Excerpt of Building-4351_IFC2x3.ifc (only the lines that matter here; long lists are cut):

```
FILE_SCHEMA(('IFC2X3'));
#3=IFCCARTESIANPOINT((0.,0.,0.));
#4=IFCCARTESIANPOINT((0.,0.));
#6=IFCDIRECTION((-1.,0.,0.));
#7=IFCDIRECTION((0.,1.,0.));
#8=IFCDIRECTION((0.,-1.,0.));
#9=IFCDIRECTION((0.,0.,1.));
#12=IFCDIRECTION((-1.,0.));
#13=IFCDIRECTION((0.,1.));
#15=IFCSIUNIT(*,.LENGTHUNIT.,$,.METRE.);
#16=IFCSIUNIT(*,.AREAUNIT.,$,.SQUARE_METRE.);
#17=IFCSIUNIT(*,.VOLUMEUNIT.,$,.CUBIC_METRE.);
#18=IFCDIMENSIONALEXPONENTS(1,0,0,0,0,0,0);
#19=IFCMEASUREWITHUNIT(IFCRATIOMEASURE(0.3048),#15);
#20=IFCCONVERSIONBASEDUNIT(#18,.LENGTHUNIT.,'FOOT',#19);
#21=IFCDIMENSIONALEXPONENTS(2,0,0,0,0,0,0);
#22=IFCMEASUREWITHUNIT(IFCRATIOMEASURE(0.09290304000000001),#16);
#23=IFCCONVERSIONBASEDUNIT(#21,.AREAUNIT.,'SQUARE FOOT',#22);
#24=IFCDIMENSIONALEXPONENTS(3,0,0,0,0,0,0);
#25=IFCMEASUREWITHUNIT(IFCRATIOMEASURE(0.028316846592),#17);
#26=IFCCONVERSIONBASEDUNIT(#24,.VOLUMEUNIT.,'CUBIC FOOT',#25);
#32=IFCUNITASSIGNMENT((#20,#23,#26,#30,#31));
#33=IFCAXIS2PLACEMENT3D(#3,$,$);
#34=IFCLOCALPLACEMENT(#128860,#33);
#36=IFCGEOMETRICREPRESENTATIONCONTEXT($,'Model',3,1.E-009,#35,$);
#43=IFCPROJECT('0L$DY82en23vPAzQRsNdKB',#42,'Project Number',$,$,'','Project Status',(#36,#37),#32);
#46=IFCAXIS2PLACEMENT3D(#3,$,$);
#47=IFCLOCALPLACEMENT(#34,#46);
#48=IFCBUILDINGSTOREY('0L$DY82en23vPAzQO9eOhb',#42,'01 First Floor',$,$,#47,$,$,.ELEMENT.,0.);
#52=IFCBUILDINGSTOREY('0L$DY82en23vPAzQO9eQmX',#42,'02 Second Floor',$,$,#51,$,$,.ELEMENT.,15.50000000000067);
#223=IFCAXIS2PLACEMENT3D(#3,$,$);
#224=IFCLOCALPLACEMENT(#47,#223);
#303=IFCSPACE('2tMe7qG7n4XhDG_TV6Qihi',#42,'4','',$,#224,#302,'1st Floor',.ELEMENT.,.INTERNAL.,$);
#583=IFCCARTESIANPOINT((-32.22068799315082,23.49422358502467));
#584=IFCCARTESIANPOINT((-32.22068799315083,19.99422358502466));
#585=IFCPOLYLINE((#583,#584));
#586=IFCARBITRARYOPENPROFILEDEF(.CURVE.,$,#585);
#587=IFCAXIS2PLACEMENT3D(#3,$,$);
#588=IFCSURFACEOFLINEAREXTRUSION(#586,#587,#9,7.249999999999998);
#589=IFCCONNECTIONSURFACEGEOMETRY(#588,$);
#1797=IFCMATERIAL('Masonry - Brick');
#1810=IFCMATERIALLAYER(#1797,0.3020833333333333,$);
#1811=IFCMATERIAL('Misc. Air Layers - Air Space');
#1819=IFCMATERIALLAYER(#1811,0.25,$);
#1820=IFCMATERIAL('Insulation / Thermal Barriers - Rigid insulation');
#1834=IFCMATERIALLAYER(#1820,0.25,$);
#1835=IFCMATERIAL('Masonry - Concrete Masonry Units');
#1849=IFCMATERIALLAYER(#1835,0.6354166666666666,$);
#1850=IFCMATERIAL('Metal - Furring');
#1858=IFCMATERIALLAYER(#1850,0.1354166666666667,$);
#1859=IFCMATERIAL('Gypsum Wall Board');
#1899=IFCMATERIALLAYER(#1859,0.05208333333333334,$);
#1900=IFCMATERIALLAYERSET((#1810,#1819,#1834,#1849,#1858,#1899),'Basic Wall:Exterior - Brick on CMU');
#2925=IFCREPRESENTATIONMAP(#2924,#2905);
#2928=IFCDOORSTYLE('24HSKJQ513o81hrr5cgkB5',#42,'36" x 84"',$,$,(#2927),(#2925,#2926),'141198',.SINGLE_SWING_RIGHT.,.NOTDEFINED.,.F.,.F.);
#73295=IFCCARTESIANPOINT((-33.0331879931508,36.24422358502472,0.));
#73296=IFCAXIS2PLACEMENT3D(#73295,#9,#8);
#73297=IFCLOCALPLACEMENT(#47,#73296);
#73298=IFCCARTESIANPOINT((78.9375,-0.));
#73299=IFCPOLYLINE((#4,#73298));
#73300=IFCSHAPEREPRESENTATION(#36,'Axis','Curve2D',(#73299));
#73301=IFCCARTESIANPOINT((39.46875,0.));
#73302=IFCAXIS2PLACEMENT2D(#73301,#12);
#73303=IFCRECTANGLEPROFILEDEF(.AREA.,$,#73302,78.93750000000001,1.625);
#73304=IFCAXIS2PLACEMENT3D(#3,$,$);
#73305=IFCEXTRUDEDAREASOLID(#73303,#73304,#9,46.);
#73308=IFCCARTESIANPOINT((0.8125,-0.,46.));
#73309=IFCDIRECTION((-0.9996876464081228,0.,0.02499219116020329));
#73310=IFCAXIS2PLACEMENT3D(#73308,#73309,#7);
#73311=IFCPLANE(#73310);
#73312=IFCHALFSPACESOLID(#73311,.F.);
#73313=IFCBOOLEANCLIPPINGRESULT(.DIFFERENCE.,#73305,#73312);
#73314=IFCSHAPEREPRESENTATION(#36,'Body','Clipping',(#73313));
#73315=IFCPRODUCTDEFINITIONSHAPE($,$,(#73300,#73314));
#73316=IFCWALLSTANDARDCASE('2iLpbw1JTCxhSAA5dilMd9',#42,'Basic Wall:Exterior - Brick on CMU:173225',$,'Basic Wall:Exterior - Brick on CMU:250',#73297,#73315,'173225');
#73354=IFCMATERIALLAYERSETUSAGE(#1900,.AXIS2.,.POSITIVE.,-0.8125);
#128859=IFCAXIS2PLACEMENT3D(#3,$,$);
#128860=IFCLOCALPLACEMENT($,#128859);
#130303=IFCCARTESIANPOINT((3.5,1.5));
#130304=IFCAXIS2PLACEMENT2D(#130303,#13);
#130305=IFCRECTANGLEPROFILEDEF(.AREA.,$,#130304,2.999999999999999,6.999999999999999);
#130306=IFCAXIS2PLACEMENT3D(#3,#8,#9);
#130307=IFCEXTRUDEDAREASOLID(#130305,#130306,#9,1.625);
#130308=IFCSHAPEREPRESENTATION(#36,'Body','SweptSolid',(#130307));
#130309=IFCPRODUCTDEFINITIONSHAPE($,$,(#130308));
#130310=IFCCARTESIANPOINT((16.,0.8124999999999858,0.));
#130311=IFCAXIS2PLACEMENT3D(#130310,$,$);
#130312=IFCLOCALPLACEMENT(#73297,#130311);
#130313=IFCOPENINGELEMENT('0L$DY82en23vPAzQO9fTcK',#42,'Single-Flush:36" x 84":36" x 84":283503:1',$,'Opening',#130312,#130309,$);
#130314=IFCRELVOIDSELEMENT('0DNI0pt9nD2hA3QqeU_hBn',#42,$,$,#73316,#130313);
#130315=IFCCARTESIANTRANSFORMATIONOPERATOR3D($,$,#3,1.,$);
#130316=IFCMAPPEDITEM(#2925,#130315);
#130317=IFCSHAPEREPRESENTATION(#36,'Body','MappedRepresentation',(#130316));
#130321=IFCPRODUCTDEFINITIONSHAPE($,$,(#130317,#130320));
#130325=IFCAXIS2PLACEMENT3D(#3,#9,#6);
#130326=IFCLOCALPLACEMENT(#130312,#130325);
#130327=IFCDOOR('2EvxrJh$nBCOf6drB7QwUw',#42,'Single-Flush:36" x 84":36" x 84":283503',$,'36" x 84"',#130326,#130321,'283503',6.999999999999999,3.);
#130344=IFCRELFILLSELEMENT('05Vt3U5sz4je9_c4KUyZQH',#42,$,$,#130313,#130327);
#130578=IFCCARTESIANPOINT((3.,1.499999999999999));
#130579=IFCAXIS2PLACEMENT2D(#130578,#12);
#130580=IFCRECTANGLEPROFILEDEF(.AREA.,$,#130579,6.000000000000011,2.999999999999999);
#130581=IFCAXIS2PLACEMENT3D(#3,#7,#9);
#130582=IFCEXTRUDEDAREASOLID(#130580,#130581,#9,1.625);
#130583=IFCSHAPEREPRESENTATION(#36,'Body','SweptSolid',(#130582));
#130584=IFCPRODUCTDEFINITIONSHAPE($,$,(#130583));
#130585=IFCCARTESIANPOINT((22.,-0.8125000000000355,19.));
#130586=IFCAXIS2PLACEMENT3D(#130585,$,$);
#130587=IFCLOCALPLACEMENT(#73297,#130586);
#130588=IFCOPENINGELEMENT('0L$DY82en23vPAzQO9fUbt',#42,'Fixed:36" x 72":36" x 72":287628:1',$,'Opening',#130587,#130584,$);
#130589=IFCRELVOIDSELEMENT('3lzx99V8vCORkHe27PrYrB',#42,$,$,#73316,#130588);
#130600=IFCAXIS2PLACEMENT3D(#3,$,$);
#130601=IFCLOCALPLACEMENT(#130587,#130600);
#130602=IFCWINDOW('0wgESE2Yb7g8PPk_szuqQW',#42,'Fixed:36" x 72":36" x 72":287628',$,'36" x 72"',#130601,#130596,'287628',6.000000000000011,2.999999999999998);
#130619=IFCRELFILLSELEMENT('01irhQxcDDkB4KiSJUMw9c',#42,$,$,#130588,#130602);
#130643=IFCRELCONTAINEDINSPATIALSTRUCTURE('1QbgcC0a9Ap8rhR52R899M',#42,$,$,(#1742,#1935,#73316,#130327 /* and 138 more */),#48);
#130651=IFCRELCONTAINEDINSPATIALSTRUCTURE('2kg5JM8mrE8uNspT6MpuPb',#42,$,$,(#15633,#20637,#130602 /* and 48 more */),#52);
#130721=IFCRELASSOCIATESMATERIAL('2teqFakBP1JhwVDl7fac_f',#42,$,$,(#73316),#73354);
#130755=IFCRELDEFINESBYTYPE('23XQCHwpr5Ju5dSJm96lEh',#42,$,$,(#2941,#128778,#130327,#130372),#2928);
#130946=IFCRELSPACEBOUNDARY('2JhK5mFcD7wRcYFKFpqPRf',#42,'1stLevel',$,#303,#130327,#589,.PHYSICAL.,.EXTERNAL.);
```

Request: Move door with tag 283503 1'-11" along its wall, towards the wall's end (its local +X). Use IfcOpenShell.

```python
import numpy as np
import ifcopenshell
import ifcopenshell.api.geometry
import ifcopenshell.util.placement
import ifcopenshell.util.unit

model = ifcopenshell.open("Building-4351_IFC2x3.ifc")
unit_scale = ifcopenshell.util.unit.calculate_unit_scale(model)

door = model.by_guid("2EvxrJh$nBCOf6drB7QwUw")
opening = door.FillsVoids[0].RelatingOpeningElement
wall = opening.VoidsElements[0].RelatingBuildingElement

wall_matrix = ifcopenshell.util.placement.get_local_placement(wall.ObjectPlacement)
shift = wall_matrix[:3, 0] * 23 * 0.0254 / unit_scale
before = ifcopenshell.util.placement.get_local_placement(door.ObjectPlacement)[:3, 3].copy()

# The door is placed relative to its opening, so it follows when the opening moves.
matrix = ifcopenshell.util.placement.get_local_placement(opening.ObjectPlacement)
matrix[:3, 3] += shift
ifcopenshell.api.geometry.edit_object_placement(
    model, product=opening, matrix=matrix, is_si=False, should_transform_children=True
)

# Space boundary surfaces are stored in each space's coordinates; move them too.
for rel in door.ProvidesBoundaries:
    if not rel.ConnectionGeometry:
        continue
    surface = rel.ConnectionGeometry.SurfaceOnRelatingElement
    space_matrix = ifcopenshell.util.placement.get_local_placement(rel.RelatingSpace.ObjectPlacement)
    point = np.array(surface.Position.Location.Coordinates) + space_matrix[:3, :3].T @ shift
    surface.Position = model.createIfcAxis2Placement3D(
        model.createIfcCartesianPoint(point.tolist()), surface.Position.Axis, surface.Position.RefDirection
    )

after = ifcopenshell.util.placement.get_local_placement(door.ObjectPlacement)[:3, 3]
print("door moved by", (after - before).round(3) + 0.0)

model.write("Building-4351_IFC2x3_v2.ifc")
```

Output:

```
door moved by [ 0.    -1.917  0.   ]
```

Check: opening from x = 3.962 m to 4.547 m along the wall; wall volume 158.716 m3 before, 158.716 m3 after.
